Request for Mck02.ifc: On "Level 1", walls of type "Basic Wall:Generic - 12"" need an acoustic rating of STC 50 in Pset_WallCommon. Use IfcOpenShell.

First a look at what the model holds.

```python
import ifcopenshell
import ifcopenshell.util.element

model = ifcopenshell.open("Mck02.ifc")
print(model.schema)
storey = next(s for s in model.by_type("IfcBuildingStorey") if s.Name == "Level 1")
walls = [e for e in ifcopenshell.util.element.get_decomposition(storey) if e.is_a("IfcWall")]
seen = {}
for e in walls:
    element_type = ifcopenshell.util.element.get_type(e)
    key = (element_type.Name if element_type != e and element_type else None, ifcopenshell.util.element.get_pset(e, "Pset_WallCommon", "AcousticRating"))
    seen[key] = seen.get(key, 0) + 1
for (name, value), count in sorted(seen.items(), key=str):
    print(count, "x", name, "|", value)
```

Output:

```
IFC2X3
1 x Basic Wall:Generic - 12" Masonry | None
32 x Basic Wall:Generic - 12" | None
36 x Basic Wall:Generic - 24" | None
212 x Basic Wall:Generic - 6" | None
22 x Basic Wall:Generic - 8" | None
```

```python
import ifcopenshell
import ifcopenshell.api.pset
import ifcopenshell.util.element

model = ifcopenshell.open("Mck02.ifc")

storey = next(s for s in model.by_type("IfcBuildingStorey") if s.Name == "Level 1")
walls = [e for e in ifcopenshell.util.element.get_decomposition(storey) if e.is_a("IfcWall")]

count = 0
for e in walls:
    element_type = ifcopenshell.util.element.get_type(e)
    if element_type in (None, e) or element_type.Name != 'Basic Wall:Generic - 12"':
        continue
    # add_pset returns the element's existing set when there is one.
    pset = ifcopenshell.api.pset.add_pset(model, product=e, name="Pset_WallCommon")
    ifcopenshell.api.pset.edit_pset(model, pset=pset, properties={"AcousticRating": "STC 50"})
    count += 1

print(count, "walls updated")

model.write("Mck02_rev.ifc")
```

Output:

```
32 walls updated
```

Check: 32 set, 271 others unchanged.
